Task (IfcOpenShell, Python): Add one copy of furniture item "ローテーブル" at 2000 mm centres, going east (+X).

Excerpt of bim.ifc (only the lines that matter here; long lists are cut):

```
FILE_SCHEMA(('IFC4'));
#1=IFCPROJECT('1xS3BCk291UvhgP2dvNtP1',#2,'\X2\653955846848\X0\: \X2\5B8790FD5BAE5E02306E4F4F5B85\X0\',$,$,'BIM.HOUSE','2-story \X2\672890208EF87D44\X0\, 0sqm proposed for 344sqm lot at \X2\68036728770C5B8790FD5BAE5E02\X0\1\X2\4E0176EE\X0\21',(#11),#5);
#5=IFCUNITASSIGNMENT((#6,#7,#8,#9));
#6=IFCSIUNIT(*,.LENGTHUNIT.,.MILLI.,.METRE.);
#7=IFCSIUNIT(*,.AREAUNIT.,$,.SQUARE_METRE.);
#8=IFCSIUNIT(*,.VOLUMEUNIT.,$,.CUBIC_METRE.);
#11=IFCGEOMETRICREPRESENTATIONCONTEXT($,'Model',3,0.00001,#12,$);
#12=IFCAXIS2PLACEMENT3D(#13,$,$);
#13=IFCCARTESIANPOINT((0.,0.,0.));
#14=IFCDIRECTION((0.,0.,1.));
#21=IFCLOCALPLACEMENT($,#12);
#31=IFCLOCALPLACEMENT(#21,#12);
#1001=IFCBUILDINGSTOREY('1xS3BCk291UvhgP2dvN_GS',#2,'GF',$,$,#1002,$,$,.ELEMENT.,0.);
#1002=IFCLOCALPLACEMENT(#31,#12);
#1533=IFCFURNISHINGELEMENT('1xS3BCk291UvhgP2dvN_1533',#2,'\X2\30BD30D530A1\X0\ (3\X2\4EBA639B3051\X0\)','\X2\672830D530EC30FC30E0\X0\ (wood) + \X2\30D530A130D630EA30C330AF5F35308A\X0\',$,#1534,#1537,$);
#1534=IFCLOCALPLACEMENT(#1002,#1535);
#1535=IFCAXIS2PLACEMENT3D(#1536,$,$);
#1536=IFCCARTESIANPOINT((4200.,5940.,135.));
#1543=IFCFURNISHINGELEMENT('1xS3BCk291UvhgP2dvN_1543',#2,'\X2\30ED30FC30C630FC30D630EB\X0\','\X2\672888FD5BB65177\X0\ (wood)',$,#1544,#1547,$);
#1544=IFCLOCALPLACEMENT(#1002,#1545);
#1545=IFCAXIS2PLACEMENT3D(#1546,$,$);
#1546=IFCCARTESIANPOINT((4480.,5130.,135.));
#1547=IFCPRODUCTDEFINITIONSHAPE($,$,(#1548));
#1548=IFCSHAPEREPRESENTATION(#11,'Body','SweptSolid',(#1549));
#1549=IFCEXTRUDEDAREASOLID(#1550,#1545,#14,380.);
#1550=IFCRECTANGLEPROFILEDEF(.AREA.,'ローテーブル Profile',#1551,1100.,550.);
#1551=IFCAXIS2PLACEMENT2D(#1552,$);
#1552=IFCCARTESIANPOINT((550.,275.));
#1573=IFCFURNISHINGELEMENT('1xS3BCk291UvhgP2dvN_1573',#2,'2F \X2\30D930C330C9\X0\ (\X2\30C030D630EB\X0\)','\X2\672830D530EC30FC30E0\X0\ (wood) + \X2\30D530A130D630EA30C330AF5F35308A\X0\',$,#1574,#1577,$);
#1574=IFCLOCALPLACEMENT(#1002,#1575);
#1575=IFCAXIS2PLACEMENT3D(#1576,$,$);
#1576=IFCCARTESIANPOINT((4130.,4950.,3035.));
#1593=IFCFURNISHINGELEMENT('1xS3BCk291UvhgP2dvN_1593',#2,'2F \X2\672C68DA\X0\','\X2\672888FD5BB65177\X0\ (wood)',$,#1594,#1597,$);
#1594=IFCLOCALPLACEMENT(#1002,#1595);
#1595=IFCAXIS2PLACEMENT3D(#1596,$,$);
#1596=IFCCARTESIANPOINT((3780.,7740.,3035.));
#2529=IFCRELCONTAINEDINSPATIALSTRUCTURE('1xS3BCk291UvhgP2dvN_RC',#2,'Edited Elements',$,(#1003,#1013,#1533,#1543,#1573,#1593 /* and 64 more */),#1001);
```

```python
import numpy as np
import ifcopenshell
import ifcopenshell.api.geometry
import ifcopenshell.api.root
import ifcopenshell.util.element
import ifcopenshell.util.placement
import ifcopenshell.util.unit

model = ifcopenshell.open("bim.ifc")
unit_scale = ifcopenshell.util.unit.calculate_unit_scale(model)


def reuse_history(source, copy):
    """copy_class also copies each property set's owner history, people and application; keep the originals."""
    for rel in copy.IsDefinedBy:
        if rel.is_a("IfcRelDefinesByProperties") and (history := rel.RelatingPropertyDefinition.OwnerHistory):
            rel.RelatingPropertyDefinition.OwnerHistory = source.OwnerHistory
            ifcopenshell.util.element.remove_deep2(model, history)


source = model.by_guid("1xS3BCk291UvhgP2dvN_1543")
base = ifcopenshell.util.placement.get_local_placement(source.ObjectPlacement)
step = np.array([1.0, 0.0, 0.0]) * 2 / unit_scale

for i in range(1, 2):
    copy = ifcopenshell.api.root.copy_class(model, product=source)
    copy.Representation = ifcopenshell.util.element.copy_deep(
        model, source.Representation, exclude=["IfcGeometricRepresentationContext", "IfcRepresentationMap"]
    )
    reuse_history(source, copy)
    matrix = base.copy()
    matrix[:3, 3] += i * step
    print("added at", matrix[:3, 3].round(3) + 0.0)
    ifcopenshell.api.geometry.edit_object_placement(model, product=copy, matrix=matrix, is_si=False)

model.write("bim-out.ifc")
```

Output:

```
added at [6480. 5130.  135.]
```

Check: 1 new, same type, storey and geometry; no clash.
